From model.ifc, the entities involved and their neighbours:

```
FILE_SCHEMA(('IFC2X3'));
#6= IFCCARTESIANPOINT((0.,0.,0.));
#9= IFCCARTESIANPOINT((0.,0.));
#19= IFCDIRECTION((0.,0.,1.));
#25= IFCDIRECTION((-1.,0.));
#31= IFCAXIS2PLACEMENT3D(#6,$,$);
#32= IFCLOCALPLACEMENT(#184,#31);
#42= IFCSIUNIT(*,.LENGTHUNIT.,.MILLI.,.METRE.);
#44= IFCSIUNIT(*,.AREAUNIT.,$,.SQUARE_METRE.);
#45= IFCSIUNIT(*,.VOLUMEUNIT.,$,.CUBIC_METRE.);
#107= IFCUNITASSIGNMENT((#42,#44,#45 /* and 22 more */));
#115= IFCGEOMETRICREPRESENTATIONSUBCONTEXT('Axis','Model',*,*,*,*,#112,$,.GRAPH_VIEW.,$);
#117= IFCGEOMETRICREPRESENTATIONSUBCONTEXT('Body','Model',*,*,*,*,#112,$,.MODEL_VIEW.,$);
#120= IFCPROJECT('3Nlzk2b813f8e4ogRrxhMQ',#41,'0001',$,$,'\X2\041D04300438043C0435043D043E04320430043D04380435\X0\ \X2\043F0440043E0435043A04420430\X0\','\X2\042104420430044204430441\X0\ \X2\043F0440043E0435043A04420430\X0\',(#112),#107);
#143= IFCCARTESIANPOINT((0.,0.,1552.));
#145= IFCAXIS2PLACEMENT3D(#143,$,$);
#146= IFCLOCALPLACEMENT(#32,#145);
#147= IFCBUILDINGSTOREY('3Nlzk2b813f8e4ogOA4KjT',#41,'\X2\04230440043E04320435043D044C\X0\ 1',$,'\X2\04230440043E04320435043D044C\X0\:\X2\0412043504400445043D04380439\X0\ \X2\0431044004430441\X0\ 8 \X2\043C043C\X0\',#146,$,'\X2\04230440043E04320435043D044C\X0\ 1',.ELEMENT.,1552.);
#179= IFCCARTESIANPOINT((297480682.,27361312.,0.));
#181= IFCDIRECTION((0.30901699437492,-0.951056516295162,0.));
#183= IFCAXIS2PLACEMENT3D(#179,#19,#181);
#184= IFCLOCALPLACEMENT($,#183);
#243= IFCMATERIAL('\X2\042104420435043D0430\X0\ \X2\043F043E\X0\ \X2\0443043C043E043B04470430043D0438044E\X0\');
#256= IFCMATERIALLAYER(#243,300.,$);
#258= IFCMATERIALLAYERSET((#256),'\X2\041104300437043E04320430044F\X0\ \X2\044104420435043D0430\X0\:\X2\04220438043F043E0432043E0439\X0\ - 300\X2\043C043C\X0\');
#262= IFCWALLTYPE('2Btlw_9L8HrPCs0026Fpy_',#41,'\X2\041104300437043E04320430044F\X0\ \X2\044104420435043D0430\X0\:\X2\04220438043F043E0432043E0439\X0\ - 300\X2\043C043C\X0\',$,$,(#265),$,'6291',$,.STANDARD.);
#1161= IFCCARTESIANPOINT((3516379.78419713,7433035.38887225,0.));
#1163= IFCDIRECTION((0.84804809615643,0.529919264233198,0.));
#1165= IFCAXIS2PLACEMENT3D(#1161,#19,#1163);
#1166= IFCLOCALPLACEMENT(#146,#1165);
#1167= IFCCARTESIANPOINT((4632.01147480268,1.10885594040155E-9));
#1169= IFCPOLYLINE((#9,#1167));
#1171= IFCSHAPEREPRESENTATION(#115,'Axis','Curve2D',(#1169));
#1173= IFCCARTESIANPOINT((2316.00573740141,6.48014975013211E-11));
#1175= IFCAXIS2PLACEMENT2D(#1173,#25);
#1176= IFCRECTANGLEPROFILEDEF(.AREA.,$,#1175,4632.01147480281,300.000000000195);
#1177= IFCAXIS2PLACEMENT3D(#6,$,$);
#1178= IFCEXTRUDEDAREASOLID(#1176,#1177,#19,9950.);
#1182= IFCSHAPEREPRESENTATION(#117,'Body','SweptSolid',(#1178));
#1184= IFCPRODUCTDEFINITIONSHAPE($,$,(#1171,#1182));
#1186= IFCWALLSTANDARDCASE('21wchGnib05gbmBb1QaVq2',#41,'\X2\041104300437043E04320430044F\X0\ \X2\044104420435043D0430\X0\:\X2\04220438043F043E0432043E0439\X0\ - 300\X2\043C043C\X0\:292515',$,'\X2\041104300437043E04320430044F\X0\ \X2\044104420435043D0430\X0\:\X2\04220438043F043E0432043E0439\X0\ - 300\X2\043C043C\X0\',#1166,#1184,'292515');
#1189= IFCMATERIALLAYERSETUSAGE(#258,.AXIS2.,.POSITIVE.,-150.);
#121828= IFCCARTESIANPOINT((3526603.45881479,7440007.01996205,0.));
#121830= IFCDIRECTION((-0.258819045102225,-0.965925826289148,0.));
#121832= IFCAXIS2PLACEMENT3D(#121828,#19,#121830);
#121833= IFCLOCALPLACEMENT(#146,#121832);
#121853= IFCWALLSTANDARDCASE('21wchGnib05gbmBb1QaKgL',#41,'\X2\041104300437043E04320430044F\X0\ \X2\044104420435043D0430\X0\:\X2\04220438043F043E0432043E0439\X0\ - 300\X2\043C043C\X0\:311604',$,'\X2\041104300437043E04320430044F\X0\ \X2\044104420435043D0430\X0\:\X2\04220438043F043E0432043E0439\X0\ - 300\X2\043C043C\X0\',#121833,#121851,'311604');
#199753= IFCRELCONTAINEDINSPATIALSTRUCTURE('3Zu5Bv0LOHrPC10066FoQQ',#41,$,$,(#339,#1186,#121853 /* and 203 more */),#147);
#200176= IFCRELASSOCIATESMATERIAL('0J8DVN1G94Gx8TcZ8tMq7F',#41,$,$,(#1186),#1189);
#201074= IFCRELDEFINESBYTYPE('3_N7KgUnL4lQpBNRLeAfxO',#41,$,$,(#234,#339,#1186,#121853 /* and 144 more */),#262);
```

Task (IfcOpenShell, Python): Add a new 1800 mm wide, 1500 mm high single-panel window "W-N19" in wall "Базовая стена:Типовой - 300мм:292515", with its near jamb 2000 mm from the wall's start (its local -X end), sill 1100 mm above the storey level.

```python
import numpy as np
import ifcopenshell
import ifcopenshell.api.feature
import ifcopenshell.api.geometry
import ifcopenshell.api.root
import ifcopenshell.api.spatial
import ifcopenshell.api.type
import ifcopenshell.geom
import ifcopenshell.util.element
import ifcopenshell.util.placement
import ifcopenshell.util.representation
import ifcopenshell.util.shape
import ifcopenshell.util.unit

model = ifcopenshell.open("model.ifc")
unit_scale = ifcopenshell.util.unit.calculate_unit_scale(model)
settings = ifcopenshell.geom.settings()


def volume(element):
    """Net volume in cubic metres, openings subtracted."""
    shape = ifcopenshell.geom.create_shape(settings, element)
    return ifcopenshell.util.shape.get_volume(shape.geometry)


wall = model.by_guid("21wchGnib05gbmBb1QaVq2")
storey = ifcopenshell.util.element.get_container(wall, ifc_class="IfcBuildingStorey")
context = ifcopenshell.util.representation.get_context(model, "Model", "Body", "MODEL_VIEW")
before = volume(wall)

width, height, from_end, sill = 1.8, 1.5, 2, 1.1  # metres

# The wall runs along its own X axis, and the end named is its -X end.
wall_shape = ifcopenshell.geom.create_shape(settings, wall)
x, y, z = ifcopenshell.util.shape.get_vertices(wall_shape.geometry).T
start = x.min() + from_end
face, thickness = float(y.min()), float(y.max() - y.min())
wall_matrix = ifcopenshell.util.placement.get_local_placement(wall.ObjectPlacement)
level = ifcopenshell.util.placement.get_local_placement(storey.ObjectPlacement)[2, 3]


def in_wall(x, y):
    """Placement at x, y metres in the wall's axes, at sill height."""
    matrix = wall_matrix.copy()
    matrix[:, 3] = wall_matrix @ np.array([x / unit_scale, y / unit_scale, 0.0, 1.0])
    matrix[2, 3] = level + sill / unit_scale
    return matrix


# Opening: a box that overshoots both wall faces by 50 mm.
opening = ifcopenshell.api.root.create_entity(model, ifc_class="IfcOpeningElement")
box = ifcopenshell.api.geometry.add_wall_representation(
    model, context=context, length=width, height=height, thickness=thickness + 0.1
)
ifcopenshell.api.geometry.assign_representation(model, product=opening, representation=box)
ifcopenshell.api.geometry.edit_object_placement(model, product=opening, matrix=in_wall(start, face - 0.05), is_si=False)
ifcopenshell.api.feature.add_feature(model, feature=opening, element=wall)

window = ifcopenshell.api.root.create_entity(model, ifc_class="IfcWindow", name="W-N19")
window.OverallWidth, window.OverallHeight = width / unit_scale, height / unit_scale
body = ifcopenshell.api.geometry.add_window_representation(
    model,
    context=context,
    overall_width=window.OverallWidth,
    overall_height=window.OverallHeight,
    partition_type="SINGLE_PANEL",
)
ifcopenshell.api.geometry.assign_representation(model, product=window, representation=body)
ifcopenshell.api.spatial.assign_container(model, products=[window], relating_structure=storey)
fills = ifcopenshell.api.feature.add_filling(model, opening=opening, element=window)
fills.OwnerHistory = window.OwnerHistory  # required in IFC2X3

# IFC2X3 keeps the operation on the window style.
style = ifcopenshell.api.root.create_entity(model, ifc_class="IfcWindowStyle", name="W-N19")
style.OperationType, style.ConstructionType = "SINGLE_PANEL", "NOTDEFINED"
style.ParameterTakesPrecedence = style.Sizeable = False
ifcopenshell.api.type.assign_type(model, related_objects=[window], relating_type=style)

# Centre the window in the wall's thickness.
ifcopenshell.api.geometry.edit_object_placement(model, product=window, matrix=in_wall(start, face), is_si=False)
window_shape = ifcopenshell.geom.create_shape(settings, window)
depth = ifcopenshell.util.shape.get_vertices(window_shape.geometry)[:, 1]
offset = face + thickness / 2 - (depth.min() + depth.max()) / 2
ifcopenshell.api.geometry.edit_object_placement(model, product=window, matrix=in_wall(start, offset), is_si=False)

after = volume(wall)

print(f"wall volume {before:.3f} -> {after:.3f} m3")

model.write("model_edited.ifc")
```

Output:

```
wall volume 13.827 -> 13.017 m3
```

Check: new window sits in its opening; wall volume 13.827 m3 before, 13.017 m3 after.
